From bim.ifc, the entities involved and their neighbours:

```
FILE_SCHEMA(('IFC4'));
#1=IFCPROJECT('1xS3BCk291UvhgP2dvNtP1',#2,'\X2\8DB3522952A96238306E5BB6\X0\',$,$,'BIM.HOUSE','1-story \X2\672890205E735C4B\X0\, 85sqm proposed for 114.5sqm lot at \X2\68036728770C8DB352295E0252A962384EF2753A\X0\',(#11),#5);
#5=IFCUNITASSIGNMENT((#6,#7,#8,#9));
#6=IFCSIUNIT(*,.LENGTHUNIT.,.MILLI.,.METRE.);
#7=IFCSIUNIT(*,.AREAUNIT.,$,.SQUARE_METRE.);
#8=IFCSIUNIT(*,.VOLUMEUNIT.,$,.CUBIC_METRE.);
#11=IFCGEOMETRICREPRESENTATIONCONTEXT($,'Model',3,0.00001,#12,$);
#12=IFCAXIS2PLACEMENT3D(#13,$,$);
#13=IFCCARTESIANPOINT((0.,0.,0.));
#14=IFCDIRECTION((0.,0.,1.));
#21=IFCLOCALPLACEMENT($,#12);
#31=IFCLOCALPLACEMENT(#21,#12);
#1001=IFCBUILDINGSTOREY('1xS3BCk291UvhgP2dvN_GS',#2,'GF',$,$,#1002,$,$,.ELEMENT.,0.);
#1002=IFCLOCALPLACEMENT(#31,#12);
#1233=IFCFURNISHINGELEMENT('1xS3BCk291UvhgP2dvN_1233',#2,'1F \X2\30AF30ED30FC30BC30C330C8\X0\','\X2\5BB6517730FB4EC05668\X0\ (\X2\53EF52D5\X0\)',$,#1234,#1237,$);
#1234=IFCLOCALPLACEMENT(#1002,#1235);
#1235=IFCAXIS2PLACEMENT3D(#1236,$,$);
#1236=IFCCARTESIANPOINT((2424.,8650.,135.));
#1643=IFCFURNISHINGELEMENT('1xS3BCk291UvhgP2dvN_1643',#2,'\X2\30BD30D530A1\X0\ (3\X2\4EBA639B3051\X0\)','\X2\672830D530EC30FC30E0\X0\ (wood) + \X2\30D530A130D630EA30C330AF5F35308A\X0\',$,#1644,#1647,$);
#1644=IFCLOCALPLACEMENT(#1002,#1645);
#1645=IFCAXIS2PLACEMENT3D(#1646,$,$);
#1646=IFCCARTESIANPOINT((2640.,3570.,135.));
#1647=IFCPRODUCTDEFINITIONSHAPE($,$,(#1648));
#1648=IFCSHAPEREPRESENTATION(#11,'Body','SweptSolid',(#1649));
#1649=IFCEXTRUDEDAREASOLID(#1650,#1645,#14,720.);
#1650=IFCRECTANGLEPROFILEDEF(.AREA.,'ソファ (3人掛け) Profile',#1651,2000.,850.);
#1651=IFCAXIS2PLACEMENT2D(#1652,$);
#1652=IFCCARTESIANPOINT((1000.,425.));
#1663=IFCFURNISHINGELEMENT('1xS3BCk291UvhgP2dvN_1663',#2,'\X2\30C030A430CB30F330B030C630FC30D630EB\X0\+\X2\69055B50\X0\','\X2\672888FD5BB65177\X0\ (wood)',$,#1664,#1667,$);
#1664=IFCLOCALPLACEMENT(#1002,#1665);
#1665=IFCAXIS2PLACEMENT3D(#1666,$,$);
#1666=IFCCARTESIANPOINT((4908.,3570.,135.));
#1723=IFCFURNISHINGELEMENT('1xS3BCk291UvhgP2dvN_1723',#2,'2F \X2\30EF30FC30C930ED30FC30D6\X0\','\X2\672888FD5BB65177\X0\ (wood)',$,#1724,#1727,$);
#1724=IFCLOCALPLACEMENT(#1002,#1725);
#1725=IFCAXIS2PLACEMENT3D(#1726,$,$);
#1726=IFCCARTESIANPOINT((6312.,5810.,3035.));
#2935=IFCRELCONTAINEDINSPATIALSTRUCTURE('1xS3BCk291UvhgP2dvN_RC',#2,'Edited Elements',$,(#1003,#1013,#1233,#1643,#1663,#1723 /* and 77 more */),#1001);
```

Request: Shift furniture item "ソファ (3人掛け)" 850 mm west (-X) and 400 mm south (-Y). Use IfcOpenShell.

```python
import ifcopenshell
import ifcopenshell.api.geometry
import ifcopenshell.util.placement

model = ifcopenshell.open("bim.ifc")

item = model.by_id(1643)
matrix = ifcopenshell.util.placement.get_local_placement(item.ObjectPlacement)
matrix[0, 3] -= 850.0
matrix[1, 3] -= 400.0
ifcopenshell.api.geometry.edit_object_placement(model, product=item, matrix=matrix, is_si=False)

print(ifcopenshell.util.placement.get_local_placement(item.ObjectPlacement).round(3) + 0.0)

model.write("bim_rev.ifc")
```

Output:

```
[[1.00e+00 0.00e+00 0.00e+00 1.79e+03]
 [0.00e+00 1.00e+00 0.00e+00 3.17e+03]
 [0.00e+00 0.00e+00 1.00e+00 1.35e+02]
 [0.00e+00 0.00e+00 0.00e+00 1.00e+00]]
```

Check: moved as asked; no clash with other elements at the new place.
